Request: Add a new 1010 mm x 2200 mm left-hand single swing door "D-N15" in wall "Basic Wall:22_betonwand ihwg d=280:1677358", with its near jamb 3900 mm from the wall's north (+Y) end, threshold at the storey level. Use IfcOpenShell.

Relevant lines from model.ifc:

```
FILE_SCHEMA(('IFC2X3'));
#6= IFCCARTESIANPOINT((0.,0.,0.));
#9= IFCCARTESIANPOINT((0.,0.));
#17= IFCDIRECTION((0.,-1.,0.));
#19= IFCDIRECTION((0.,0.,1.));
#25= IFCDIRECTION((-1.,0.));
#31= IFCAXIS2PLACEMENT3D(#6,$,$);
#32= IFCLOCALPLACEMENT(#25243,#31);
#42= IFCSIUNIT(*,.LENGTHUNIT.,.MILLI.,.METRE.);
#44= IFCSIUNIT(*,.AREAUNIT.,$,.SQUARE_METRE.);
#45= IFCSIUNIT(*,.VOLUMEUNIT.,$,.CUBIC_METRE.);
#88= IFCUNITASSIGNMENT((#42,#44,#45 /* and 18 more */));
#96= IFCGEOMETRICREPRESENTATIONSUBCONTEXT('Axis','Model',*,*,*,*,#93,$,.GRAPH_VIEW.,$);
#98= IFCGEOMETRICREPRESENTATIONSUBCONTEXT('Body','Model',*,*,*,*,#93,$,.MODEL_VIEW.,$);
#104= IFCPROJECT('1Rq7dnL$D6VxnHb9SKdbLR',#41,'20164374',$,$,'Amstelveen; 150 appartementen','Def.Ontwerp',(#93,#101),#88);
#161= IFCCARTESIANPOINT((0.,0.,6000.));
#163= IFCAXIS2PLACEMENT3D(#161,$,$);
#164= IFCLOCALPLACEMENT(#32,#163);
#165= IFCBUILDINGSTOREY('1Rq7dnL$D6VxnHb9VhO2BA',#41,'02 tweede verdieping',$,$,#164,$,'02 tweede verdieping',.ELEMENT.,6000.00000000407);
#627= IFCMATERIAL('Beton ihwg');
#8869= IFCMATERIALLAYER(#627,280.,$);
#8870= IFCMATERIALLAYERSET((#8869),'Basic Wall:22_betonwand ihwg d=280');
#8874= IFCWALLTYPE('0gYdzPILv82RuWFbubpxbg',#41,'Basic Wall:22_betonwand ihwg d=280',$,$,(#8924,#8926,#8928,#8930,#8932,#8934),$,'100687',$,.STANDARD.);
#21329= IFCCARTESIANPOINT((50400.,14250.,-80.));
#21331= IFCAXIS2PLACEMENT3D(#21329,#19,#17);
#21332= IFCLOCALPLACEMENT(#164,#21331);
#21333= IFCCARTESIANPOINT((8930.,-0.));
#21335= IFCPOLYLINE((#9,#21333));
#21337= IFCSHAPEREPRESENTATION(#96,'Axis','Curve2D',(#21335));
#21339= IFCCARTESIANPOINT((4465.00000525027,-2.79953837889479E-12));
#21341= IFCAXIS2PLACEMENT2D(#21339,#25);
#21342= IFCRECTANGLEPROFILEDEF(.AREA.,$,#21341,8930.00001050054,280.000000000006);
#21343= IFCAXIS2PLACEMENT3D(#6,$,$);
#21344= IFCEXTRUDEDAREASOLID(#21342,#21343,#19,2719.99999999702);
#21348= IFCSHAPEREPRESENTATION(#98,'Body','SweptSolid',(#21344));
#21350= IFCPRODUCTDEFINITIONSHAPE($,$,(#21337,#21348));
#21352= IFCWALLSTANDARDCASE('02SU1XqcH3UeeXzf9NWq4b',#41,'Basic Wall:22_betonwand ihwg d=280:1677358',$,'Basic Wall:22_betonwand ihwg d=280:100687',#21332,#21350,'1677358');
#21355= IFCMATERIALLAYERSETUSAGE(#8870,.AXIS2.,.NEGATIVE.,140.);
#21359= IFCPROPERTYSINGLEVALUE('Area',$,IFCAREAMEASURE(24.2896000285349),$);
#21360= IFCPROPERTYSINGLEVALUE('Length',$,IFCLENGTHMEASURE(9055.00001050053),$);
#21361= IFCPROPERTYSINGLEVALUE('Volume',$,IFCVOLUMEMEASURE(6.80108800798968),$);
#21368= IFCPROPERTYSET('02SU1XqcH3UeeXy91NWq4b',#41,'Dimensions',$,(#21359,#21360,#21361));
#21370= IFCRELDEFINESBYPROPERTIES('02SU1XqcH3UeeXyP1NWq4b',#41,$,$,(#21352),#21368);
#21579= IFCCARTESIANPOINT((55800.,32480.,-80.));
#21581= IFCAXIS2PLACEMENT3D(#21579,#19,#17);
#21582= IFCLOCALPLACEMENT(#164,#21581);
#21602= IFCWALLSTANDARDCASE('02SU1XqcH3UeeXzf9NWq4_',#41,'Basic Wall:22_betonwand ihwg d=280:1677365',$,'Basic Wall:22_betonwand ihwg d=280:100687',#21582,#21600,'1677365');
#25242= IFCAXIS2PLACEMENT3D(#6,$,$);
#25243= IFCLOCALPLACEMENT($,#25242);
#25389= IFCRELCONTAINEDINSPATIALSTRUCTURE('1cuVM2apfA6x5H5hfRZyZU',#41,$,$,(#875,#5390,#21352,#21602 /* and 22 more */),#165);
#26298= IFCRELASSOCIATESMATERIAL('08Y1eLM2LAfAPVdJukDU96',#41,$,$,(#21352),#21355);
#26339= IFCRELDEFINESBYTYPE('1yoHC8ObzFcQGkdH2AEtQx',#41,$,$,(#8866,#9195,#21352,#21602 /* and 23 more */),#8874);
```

```python
import numpy as np
import ifcopenshell
import ifcopenshell.api.feature
import ifcopenshell.api.geometry
import ifcopenshell.api.pset
import ifcopenshell.api.root
import ifcopenshell.api.spatial
import ifcopenshell.api.type
import ifcopenshell.geom
import ifcopenshell.util.element
import ifcopenshell.util.placement
import ifcopenshell.util.representation
import ifcopenshell.util.shape
import ifcopenshell.util.unit

model = ifcopenshell.open("model.ifc")
unit_scale = ifcopenshell.util.unit.calculate_unit_scale(model)
area_scale = ifcopenshell.util.unit.calculate_unit_scale(model, "AREAUNIT")
volume_scale = ifcopenshell.util.unit.calculate_unit_scale(model, "VOLUMEUNIT")
settings = ifcopenshell.geom.settings()


def volume(element):
    """Net volume in cubic metres, openings subtracted."""
    shape = ifcopenshell.geom.create_shape(settings, element)
    return ifcopenshell.util.shape.get_volume(shape.geometry)


wall = model.by_id(21352)
storey = ifcopenshell.util.element.get_container(wall, ifc_class="IfcBuildingStorey")
context = ifcopenshell.util.representation.get_context(model, "Model", "Body", "MODEL_VIEW")
before = volume(wall)

width, height, from_end, sill = 1.01, 2.2, 3.9, 0.0  # metres

# The wall runs along its own X axis, and the end named is its -X end.
wall_shape = ifcopenshell.geom.create_shape(settings, wall)
x, y, z = ifcopenshell.util.shape.get_vertices(wall_shape.geometry).T
start = x.min() + from_end
face, thickness = float(y.min()), float(y.max() - y.min())
wall_matrix = ifcopenshell.util.placement.get_local_placement(wall.ObjectPlacement)
level = ifcopenshell.util.placement.get_local_placement(storey.ObjectPlacement)[2, 3]


def in_wall(x, y):
    """Placement at x, y metres in the wall's axes, at sill height."""
    matrix = wall_matrix.copy()
    matrix[:, 3] = wall_matrix @ np.array([x / unit_scale, y / unit_scale, 0.0, 1.0])
    matrix[2, 3] = level + sill / unit_scale
    return matrix


# Opening: a box that overshoots both wall faces by 50 mm.
opening = ifcopenshell.api.root.create_entity(model, ifc_class="IfcOpeningElement")
box = ifcopenshell.api.geometry.add_wall_representation(
    model, context=context, length=width, height=height, thickness=thickness + 0.1
)
ifcopenshell.api.geometry.assign_representation(model, product=opening, representation=box)
ifcopenshell.api.geometry.edit_object_placement(model, product=opening, matrix=in_wall(start, face - 0.05), is_si=False)
ifcopenshell.api.feature.add_feature(model, feature=opening, element=wall)

door = ifcopenshell.api.root.create_entity(model, ifc_class="IfcDoor", name="D-N15")
door.OverallWidth, door.OverallHeight = width / unit_scale, height / unit_scale
body = ifcopenshell.api.geometry.add_door_representation(
    model,
    context=context,
    overall_width=door.OverallWidth,
    overall_height=door.OverallHeight,
    operation_type="SINGLE_SWING_LEFT",
    lining_properties={"LiningDepth": thickness / unit_scale, "ThresholdDepth": thickness / unit_scale},
)
ifcopenshell.api.geometry.assign_representation(model, product=door, representation=body)
ifcopenshell.api.spatial.assign_container(model, products=[door], relating_structure=storey)
fills = ifcopenshell.api.feature.add_filling(model, opening=opening, element=door)
fills.OwnerHistory = door.OwnerHistory  # required in IFC2X3

# IFC2X3 keeps the operation on the door style.
style = ifcopenshell.api.root.create_entity(model, ifc_class="IfcDoorStyle", name="D-N15")
style.OperationType, style.ConstructionType = "SINGLE_SWING_LEFT", "NOTDEFINED"
style.ParameterTakesPrecedence = style.Sizeable = False
ifcopenshell.api.type.assign_type(model, related_objects=[door], relating_type=style)

# The lining spans the wall, so the door starts at the wall face.
ifcopenshell.api.geometry.edit_object_placement(model, product=door, matrix=in_wall(start, face), is_si=False)

after = volume(wall)

# Update the wall's stored quantities.
pset = model.by_id(ifcopenshell.util.element.get_pset(wall, "Dimensions", should_inherit=False)["id"])
ifcopenshell.api.pset.edit_pset(model, pset=pset, properties={
    "Area": model.create_entity("IfcAreaMeasure", after / thickness / area_scale),
    "Volume": model.create_entity("IfcVolumeMeasure", after / volume_scale),
})

print(f"wall volume {before:.3f} -> {after:.3f} m3")

model.write("model_updated.ifc")
```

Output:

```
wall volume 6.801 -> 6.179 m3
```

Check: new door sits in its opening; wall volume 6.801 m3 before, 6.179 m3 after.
